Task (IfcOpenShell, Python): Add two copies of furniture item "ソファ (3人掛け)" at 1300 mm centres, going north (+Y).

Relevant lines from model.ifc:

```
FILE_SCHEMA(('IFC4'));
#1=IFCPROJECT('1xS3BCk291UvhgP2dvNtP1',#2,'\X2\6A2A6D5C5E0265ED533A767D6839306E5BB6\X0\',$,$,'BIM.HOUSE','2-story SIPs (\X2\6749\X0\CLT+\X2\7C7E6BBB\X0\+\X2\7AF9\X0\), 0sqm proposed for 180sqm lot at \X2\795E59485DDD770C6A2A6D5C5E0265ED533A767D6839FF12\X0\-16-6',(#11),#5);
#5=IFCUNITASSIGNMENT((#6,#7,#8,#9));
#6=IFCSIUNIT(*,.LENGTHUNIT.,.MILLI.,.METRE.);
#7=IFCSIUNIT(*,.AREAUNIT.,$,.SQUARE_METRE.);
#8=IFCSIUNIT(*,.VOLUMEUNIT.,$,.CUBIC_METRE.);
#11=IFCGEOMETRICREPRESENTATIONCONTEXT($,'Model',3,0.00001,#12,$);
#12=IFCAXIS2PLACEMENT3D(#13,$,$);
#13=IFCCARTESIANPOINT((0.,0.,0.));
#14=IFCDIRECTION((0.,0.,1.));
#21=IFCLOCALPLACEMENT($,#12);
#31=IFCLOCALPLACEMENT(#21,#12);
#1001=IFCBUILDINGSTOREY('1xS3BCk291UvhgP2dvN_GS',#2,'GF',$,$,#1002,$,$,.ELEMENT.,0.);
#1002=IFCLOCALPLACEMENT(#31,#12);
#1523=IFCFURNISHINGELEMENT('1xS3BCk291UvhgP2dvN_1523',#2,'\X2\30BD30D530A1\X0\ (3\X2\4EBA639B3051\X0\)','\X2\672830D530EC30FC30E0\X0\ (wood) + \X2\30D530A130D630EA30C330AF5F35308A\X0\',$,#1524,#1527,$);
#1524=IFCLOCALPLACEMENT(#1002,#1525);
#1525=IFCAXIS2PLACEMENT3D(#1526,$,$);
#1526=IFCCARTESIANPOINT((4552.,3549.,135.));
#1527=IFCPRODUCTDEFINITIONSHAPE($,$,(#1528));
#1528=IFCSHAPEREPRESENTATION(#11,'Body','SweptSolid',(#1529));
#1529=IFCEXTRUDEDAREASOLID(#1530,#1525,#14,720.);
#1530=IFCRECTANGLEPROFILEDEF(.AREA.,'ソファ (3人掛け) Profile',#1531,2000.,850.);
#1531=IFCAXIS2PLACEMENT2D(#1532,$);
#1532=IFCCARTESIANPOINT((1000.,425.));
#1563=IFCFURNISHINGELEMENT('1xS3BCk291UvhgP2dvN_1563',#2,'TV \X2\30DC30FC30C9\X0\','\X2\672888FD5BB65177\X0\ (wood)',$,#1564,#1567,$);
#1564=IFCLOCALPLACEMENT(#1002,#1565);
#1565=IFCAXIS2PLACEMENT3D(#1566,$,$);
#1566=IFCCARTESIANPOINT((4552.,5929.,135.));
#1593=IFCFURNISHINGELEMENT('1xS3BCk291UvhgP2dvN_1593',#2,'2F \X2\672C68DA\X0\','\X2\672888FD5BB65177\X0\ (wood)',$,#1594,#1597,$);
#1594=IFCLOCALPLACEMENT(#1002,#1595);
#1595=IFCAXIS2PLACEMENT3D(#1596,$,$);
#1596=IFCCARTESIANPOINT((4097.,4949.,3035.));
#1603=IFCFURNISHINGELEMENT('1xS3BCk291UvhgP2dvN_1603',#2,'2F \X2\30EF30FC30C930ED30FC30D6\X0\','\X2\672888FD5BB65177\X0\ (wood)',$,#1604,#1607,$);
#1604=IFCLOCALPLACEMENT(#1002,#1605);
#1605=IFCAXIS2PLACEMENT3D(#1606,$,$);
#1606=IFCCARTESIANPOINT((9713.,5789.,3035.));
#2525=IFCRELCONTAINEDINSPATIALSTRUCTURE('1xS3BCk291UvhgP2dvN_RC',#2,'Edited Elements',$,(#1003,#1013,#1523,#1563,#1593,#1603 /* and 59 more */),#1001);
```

```python
import numpy as np
import ifcopenshell
import ifcopenshell.api.geometry
import ifcopenshell.api.root
import ifcopenshell.util.element
import ifcopenshell.util.placement

model = ifcopenshell.open("model.ifc")


def reuse_history(source, copy):
    """copy_class also copies each property set's owner history, people and application; keep the originals."""
    for rel in copy.IsDefinedBy:
        if rel.is_a("IfcRelDefinesByProperties") and (history := rel.RelatingPropertyDefinition.OwnerHistory):
            rel.RelatingPropertyDefinition.OwnerHistory = source.OwnerHistory
            ifcopenshell.util.element.remove_deep2(model, history)


source = model.by_guid("1xS3BCk291UvhgP2dvN_1523")
base = ifcopenshell.util.placement.get_local_placement(source.ObjectPlacement)
step = np.array([0.0, 1.0, 0.0]) * 1300.0

for i in range(1, 3):
    copy = ifcopenshell.api.root.copy_class(model, product=source)
    copy.Representation = ifcopenshell.util.element.copy_deep(
        model, source.Representation, exclude=["IfcGeometricRepresentationContext", "IfcRepresentationMap"]
    )
    reuse_history(source, copy)
    matrix = base.copy()
    matrix[:3, 3] += i * step
    print("added at", matrix[:3, 3].round(3) + 0.0)
    ifcopenshell.api.geometry.edit_object_placement(model, product=copy, matrix=matrix, is_si=False)

model.write("model_updated.ifc")
```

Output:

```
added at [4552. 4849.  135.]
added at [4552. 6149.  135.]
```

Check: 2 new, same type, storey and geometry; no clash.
